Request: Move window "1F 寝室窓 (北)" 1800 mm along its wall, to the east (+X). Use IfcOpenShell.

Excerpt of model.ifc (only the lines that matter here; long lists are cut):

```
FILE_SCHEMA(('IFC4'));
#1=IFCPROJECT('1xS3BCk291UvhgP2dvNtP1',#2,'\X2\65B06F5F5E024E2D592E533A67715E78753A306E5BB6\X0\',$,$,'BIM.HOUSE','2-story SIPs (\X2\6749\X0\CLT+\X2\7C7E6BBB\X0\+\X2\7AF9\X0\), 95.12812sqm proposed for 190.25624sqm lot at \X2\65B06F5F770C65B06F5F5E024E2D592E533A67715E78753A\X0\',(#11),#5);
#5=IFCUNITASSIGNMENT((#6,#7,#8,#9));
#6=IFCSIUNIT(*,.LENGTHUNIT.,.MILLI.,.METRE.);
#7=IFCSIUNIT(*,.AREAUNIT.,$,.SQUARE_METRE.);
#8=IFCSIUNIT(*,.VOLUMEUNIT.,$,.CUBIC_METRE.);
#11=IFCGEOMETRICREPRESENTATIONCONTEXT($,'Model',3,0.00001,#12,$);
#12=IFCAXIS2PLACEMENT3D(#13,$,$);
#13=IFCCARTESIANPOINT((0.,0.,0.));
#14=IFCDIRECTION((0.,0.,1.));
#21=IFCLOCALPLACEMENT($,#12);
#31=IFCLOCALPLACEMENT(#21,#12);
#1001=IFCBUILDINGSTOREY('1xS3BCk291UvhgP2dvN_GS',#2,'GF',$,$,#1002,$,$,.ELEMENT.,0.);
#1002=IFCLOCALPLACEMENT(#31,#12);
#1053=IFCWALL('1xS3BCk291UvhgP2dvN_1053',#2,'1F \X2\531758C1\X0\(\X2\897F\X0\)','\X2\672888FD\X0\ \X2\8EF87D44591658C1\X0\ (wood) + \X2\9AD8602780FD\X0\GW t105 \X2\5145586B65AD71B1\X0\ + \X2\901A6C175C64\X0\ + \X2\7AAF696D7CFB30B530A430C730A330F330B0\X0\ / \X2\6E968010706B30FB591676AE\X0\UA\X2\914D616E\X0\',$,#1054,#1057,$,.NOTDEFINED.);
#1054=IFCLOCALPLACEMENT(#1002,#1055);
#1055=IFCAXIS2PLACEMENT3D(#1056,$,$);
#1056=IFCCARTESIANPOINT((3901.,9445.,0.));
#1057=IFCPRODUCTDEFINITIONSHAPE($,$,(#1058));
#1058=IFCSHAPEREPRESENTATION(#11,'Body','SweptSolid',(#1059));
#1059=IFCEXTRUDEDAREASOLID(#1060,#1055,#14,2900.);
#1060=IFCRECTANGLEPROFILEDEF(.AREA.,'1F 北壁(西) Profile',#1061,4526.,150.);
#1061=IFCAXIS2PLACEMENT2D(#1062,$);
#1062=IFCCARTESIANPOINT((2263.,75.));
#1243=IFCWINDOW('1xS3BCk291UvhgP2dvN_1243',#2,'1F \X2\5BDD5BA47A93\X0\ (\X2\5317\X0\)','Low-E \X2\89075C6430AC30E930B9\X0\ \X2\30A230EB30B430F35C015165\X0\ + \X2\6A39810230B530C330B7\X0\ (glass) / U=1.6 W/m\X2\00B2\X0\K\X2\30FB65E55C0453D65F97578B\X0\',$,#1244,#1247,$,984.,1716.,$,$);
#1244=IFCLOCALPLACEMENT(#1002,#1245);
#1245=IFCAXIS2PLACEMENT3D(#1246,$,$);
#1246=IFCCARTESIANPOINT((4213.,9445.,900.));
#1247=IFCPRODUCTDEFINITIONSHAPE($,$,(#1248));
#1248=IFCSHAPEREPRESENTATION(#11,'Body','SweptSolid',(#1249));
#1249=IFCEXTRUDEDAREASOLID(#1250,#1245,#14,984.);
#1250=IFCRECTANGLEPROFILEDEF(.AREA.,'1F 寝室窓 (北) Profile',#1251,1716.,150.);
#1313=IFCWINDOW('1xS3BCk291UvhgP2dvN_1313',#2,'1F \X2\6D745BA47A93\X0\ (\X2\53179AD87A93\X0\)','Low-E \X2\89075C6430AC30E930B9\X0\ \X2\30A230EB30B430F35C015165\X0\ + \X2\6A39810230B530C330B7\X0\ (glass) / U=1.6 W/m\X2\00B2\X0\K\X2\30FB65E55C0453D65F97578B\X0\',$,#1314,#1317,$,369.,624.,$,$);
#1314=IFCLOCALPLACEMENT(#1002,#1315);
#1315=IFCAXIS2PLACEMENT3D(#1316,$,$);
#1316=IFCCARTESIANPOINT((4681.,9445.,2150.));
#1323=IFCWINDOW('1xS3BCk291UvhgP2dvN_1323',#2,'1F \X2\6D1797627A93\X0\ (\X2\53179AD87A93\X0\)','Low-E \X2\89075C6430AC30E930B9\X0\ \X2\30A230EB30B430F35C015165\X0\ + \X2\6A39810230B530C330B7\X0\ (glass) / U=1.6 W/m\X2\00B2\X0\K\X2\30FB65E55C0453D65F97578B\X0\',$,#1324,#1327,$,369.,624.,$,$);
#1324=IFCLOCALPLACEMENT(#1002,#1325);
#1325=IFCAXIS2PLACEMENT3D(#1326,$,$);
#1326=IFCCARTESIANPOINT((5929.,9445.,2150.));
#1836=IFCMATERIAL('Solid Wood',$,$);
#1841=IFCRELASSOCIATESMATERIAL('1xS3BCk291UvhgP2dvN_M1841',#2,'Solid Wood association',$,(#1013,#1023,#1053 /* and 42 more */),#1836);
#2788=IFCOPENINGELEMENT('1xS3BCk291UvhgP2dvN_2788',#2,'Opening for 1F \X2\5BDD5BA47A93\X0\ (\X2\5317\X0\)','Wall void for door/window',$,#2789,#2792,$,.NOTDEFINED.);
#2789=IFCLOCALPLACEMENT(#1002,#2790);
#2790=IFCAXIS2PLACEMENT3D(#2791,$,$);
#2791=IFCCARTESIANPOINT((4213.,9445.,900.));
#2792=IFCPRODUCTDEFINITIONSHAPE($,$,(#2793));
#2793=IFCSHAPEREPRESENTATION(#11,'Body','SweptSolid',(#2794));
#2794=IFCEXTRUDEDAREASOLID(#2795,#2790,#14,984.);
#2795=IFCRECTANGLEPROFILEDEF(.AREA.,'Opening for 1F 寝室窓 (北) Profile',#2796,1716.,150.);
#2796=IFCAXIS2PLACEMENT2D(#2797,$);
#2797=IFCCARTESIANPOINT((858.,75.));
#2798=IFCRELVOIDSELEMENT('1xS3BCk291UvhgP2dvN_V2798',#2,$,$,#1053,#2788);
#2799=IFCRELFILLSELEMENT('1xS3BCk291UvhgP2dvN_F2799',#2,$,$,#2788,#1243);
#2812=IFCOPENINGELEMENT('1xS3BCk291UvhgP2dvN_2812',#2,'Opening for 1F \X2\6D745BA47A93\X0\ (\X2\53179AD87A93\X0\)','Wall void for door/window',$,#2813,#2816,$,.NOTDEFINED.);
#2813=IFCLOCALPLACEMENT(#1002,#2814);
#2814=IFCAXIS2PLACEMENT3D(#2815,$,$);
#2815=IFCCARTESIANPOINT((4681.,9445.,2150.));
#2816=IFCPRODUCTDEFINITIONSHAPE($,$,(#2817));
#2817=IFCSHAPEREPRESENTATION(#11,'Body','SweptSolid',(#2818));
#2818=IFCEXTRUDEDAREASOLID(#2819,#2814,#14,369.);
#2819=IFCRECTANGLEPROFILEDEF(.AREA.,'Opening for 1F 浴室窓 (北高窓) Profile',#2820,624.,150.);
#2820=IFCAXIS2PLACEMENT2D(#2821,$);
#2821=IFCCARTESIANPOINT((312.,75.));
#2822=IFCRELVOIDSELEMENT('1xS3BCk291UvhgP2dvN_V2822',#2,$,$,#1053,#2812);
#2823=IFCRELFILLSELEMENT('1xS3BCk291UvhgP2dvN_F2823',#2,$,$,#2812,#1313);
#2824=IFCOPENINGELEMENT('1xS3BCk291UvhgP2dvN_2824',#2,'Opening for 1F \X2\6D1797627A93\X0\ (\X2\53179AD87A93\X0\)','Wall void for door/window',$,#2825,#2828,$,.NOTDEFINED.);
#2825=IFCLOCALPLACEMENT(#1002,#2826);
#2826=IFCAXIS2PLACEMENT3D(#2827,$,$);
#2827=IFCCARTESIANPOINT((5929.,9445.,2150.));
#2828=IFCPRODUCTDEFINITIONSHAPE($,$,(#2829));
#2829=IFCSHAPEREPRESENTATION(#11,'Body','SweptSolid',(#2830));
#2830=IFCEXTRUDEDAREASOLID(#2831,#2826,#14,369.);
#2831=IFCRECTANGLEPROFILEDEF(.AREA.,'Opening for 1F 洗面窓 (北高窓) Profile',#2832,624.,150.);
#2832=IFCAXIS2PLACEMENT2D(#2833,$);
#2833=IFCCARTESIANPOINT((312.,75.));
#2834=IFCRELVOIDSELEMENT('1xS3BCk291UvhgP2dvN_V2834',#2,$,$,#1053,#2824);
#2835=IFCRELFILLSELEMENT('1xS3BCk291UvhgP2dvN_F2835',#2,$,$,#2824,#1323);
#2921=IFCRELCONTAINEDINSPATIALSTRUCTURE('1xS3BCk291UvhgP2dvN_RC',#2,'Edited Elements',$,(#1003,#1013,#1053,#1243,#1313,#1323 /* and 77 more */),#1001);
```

```python
import ifcopenshell
import ifcopenshell.api.geometry
import ifcopenshell.util.placement
import ifcopenshell.util.unit

model = ifcopenshell.open("model.ifc")
unit_scale = ifcopenshell.util.unit.calculate_unit_scale(model)

window = model.by_id(1243)
opening = window.FillsVoids[0].RelatingOpeningElement
wall = opening.VoidsElements[0].RelatingBuildingElement

wall_matrix = ifcopenshell.util.placement.get_local_placement(wall.ObjectPlacement)
shift = wall_matrix[:3, 0] * 1.8 / unit_scale
before = ifcopenshell.util.placement.get_local_placement(window.ObjectPlacement)[:3, 3].copy()

# The window is not placed relative to its opening, so move both.
for product in (opening, window):
    matrix = ifcopenshell.util.placement.get_local_placement(product.ObjectPlacement)
    matrix[:3, 3] += shift
    ifcopenshell.api.geometry.edit_object_placement(model, product=product, matrix=matrix, is_si=False)

after = ifcopenshell.util.placement.get_local_placement(window.ObjectPlacement)[:3, 3]
print("window moved by", (after - before).round(3) + 0.0)

model.write("model_rev.ifc")
```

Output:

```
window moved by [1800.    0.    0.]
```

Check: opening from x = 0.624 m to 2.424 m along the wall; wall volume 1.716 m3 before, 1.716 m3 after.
